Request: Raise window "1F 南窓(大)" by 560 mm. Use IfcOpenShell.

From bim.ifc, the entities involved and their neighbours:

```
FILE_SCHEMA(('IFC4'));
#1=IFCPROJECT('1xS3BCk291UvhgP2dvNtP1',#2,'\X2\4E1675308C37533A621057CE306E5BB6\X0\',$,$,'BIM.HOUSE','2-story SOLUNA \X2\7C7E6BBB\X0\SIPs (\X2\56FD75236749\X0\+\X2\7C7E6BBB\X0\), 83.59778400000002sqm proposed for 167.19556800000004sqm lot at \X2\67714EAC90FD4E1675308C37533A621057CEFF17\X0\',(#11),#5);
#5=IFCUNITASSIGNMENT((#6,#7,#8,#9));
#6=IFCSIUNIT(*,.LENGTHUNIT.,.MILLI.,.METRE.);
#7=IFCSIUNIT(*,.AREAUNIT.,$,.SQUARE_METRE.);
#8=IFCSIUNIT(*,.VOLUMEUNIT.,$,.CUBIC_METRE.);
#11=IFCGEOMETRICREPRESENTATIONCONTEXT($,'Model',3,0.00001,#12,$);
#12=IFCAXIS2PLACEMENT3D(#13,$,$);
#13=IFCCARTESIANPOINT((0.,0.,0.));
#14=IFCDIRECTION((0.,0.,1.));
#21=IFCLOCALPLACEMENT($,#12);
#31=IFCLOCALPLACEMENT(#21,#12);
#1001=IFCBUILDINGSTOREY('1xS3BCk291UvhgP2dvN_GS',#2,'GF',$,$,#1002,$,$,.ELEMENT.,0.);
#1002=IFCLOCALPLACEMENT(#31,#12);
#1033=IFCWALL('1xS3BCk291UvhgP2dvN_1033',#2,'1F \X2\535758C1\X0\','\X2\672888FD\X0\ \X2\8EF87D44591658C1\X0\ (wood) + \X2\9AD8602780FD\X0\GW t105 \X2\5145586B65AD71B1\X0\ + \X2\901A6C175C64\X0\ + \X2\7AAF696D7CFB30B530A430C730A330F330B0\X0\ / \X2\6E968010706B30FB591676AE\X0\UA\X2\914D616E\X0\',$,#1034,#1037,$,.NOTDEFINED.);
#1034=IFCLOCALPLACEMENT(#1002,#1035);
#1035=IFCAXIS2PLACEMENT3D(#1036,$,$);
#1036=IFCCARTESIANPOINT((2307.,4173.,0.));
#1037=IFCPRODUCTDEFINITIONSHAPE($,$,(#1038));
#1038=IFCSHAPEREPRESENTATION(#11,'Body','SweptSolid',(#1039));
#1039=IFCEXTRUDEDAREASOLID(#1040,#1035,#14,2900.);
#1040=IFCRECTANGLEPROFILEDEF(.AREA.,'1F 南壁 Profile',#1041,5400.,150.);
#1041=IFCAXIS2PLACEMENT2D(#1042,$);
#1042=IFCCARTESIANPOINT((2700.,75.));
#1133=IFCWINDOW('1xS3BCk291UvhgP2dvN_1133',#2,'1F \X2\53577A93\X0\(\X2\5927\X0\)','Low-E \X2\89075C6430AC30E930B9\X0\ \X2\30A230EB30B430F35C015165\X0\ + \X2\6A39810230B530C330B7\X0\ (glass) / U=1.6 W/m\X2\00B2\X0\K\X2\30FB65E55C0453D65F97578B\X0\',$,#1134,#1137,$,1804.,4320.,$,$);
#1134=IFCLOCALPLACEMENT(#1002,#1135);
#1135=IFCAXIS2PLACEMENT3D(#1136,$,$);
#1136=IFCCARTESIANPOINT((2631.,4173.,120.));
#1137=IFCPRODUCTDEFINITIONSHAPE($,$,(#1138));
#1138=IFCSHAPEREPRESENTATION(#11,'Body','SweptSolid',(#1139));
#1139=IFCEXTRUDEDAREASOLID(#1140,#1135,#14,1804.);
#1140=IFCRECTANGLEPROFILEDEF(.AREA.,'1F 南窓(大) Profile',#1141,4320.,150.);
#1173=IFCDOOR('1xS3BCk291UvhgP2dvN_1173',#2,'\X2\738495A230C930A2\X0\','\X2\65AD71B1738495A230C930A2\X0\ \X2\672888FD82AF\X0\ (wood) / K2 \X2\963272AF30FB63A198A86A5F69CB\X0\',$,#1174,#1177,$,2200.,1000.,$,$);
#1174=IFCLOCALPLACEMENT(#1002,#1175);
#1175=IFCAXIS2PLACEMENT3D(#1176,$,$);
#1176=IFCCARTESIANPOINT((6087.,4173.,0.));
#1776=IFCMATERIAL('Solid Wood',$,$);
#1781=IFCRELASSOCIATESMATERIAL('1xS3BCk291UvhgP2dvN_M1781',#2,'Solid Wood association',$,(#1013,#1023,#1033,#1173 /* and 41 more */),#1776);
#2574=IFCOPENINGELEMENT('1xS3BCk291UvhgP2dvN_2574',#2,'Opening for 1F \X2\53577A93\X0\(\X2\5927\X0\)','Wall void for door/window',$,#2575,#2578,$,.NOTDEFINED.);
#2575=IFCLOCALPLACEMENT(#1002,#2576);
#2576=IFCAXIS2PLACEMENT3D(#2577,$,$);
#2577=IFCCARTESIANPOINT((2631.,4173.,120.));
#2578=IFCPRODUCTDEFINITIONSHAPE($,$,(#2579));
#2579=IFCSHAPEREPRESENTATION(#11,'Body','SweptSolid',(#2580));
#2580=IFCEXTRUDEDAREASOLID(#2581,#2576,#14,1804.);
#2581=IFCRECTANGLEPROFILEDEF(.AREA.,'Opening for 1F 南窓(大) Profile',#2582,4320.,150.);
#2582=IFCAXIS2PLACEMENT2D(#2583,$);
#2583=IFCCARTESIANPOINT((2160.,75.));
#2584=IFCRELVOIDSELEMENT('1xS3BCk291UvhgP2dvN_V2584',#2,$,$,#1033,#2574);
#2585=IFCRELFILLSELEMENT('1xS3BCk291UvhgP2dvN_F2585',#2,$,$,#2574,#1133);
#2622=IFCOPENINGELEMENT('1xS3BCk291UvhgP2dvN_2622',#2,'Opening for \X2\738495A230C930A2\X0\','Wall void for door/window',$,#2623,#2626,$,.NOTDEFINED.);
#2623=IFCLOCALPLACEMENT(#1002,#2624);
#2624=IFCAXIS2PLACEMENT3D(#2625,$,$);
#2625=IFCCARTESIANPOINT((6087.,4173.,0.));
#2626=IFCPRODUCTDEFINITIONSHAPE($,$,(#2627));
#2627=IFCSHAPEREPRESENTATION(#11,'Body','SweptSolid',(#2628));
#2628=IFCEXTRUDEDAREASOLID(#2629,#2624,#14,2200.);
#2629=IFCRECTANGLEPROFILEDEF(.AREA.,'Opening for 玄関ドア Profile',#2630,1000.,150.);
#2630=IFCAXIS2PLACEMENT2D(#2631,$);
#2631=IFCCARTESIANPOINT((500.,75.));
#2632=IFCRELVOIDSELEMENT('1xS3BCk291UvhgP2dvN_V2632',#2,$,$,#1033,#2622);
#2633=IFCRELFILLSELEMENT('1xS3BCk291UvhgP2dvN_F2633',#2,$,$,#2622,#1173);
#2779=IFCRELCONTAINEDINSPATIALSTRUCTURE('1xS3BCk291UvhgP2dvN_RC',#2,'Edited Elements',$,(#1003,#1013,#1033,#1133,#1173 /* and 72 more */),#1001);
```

```python
import numpy as np
import ifcopenshell
import ifcopenshell.api.geometry
import ifcopenshell.util.placement
import ifcopenshell.util.unit

model = ifcopenshell.open("bim.ifc")
unit_scale = ifcopenshell.util.unit.calculate_unit_scale(model)

window = model.by_guid("1xS3BCk291UvhgP2dvN_1133")
opening = window.FillsVoids[0].RelatingOpeningElement
dz = 560.0

shift = np.array([0.0, 0.0, dz])
# The window is not placed relative to its opening, so move both.
for product in (opening, window):
    matrix = ifcopenshell.util.placement.get_local_placement(product.ObjectPlacement)
    matrix[:3, 3] += shift
    ifcopenshell.api.geometry.edit_object_placement(model, product=product, matrix=matrix, is_si=False)

print(f"moved by {dz * unit_scale:+.3f} m")

model.write("bim_rev.ifc")
```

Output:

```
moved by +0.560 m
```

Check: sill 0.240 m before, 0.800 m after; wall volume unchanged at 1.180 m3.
